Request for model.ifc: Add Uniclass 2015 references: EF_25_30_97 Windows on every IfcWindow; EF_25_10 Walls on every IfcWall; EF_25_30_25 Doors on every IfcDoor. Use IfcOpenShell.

First a look at what the model holds.

```python
import ifcopenshell

model = ifcopenshell.open("model.ifc")
print(model.schema)
print("classifications:", [c.Name for c in model.by_type("IfcClassification")])
for ifc_class in ("IfcDoor", "IfcRoof", "IfcStair", "IfcWall", "IfcWindow"):
    print(ifc_class, len(model.by_type(ifc_class)))
```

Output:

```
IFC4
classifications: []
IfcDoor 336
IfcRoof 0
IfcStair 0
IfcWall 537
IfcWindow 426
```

```python
import ifcopenshell
import ifcopenshell.api.classification

model = ifcopenshell.open("model.ifc")

system = ifcopenshell.api.classification.add_classification(model, classification="Uniclass 2015")

codes = {
    "IfcWindow": ("EF_25_30_97", "Windows"),
    "IfcWall": ("EF_25_10", "Walls"),
    "IfcDoor": ("EF_25_30_25", "Doors"),
}
for ifc_class, (code, name) in codes.items():
    products = model.by_type(ifc_class)
    ifcopenshell.api.classification.add_reference(
        model, products=products, classification=system, identification=code, name=name
    )
    print(code, len(products))

model.write("model_edited.ifc")
```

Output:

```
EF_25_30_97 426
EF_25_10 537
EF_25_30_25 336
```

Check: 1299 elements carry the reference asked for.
